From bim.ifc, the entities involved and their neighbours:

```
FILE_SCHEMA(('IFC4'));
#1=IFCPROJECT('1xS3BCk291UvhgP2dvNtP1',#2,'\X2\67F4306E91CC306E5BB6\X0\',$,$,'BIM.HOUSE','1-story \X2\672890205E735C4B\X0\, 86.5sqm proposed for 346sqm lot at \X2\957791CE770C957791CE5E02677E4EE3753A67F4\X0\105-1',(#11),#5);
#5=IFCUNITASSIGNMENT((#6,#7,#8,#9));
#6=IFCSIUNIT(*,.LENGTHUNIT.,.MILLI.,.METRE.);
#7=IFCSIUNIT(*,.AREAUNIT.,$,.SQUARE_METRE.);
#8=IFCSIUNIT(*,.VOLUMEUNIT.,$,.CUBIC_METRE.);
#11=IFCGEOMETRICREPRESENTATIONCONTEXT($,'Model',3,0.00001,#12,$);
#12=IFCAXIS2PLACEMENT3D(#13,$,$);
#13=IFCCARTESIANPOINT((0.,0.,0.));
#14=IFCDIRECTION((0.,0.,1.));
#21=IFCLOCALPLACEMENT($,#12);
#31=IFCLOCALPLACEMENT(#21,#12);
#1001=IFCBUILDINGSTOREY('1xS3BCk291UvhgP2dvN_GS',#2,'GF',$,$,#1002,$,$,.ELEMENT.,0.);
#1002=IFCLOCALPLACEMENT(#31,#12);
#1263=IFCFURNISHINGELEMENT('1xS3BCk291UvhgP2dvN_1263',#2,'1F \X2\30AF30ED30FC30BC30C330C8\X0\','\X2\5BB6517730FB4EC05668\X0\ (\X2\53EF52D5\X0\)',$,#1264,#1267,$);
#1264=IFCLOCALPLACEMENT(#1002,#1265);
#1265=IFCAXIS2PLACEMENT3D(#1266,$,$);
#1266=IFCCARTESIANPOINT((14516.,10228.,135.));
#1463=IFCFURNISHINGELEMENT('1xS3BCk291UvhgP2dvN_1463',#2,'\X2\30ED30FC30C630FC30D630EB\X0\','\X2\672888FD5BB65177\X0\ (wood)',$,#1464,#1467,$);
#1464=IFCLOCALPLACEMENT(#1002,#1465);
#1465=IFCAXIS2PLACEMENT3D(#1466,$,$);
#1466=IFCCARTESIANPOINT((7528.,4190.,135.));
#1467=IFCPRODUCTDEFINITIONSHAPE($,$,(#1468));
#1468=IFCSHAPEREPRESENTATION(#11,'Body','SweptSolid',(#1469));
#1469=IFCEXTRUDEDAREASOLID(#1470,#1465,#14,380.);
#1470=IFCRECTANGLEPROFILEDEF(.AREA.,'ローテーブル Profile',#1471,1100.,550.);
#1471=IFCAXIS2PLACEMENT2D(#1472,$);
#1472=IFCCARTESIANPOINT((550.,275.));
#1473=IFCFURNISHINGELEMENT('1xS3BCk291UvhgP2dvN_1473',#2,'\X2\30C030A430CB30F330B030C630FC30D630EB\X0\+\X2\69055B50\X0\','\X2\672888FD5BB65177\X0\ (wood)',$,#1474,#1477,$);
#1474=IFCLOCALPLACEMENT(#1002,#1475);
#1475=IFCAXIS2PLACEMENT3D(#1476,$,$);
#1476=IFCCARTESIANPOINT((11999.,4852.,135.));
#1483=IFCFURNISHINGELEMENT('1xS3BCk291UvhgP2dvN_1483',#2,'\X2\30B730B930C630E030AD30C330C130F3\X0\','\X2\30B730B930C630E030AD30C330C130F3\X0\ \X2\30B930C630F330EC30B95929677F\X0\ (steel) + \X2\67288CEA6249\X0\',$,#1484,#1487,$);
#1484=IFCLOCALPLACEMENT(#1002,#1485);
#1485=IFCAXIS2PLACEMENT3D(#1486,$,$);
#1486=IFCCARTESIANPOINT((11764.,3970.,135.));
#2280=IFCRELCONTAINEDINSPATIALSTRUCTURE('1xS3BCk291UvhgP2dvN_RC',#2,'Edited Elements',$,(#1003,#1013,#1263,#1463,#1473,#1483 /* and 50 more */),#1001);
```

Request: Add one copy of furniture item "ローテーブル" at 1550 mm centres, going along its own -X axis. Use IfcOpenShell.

```python
import ifcopenshell
import ifcopenshell.api.geometry
import ifcopenshell.api.root
import ifcopenshell.util.element
import ifcopenshell.util.placement
import ifcopenshell.util.unit

model = ifcopenshell.open("bim.ifc")
unit_scale = ifcopenshell.util.unit.calculate_unit_scale(model)


def reuse_history(source, copy):
    """copy_class also copies each property set's owner history, people and application; keep the originals."""
    for rel in copy.IsDefinedBy:
        if rel.is_a("IfcRelDefinesByProperties") and (history := rel.RelatingPropertyDefinition.OwnerHistory):
            rel.RelatingPropertyDefinition.OwnerHistory = source.OwnerHistory
            ifcopenshell.util.element.remove_deep2(model, history)


source = model.by_guid("1xS3BCk291UvhgP2dvN_1463")
base = ifcopenshell.util.placement.get_local_placement(source.ObjectPlacement)
step = -base[:3, 0] * 1.55 / unit_scale

for i in range(1, 2):
    copy = ifcopenshell.api.root.copy_class(model, product=source)
    copy.Representation = ifcopenshell.util.element.copy_deep(
        model, source.Representation, exclude=["IfcGeometricRepresentationContext", "IfcRepresentationMap"]
    )
    reuse_history(source, copy)
    matrix = base.copy()
    matrix[:3, 3] += i * step
    print("added at", matrix[:3, 3].round(3) + 0.0)
    ifcopenshell.api.geometry.edit_object_placement(model, product=copy, matrix=matrix, is_si=False)

model.write("bim_v2.ifc")
```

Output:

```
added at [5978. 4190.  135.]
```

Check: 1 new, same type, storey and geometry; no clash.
